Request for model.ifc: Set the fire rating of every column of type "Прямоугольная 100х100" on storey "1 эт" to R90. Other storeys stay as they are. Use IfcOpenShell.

First a look at what the model holds.

```python
import ifcopenshell
import ifcopenshell.util.element

model = ifcopenshell.open("model.ifc")
print(model.schema)
storey = next(s for s in model.by_type("IfcBuildingStorey") if s.Name == "1 эт")
columns = [e for e in ifcopenshell.util.element.get_decomposition(storey) if e.is_a("IfcColumn")]
seen = {}
for e in columns:
    element_type = ifcopenshell.util.element.get_type(e)
    key = (element_type.Name if element_type != e and element_type else None, ifcopenshell.util.element.get_pset(e, "Pset_ColumnCommon", "FireRating"))
    seen[key] = seen.get(key, 0) + 1
for (name, value), count in sorted(seen.items(), key=str):
    print(count, "x", name, "|", value)
```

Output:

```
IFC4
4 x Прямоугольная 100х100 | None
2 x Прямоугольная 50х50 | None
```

```python
import ifcopenshell
import ifcopenshell.api.pset
import ifcopenshell.util.element

model = ifcopenshell.open("model.ifc")

storey = next(s for s in model.by_type("IfcBuildingStorey") if s.Name == "1 эт")
columns = [e for e in ifcopenshell.util.element.get_decomposition(storey) if e.is_a("IfcColumn")]

count = 0
for e in columns:
    element_type = ifcopenshell.util.element.get_type(e)
    if element_type in (None, e) or element_type.Name != "Прямоугольная 100х100":
        continue
    # add_pset returns the element's existing set when there is one.
    pset = ifcopenshell.api.pset.add_pset(model, product=e, name="Pset_ColumnCommon")
    ifcopenshell.api.pset.edit_pset(model, pset=pset, properties={"FireRating": "R90"})
    count += 1

print(count, "columns updated")

model.write("model_edited.ifc")
```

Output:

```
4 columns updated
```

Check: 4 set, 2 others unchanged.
